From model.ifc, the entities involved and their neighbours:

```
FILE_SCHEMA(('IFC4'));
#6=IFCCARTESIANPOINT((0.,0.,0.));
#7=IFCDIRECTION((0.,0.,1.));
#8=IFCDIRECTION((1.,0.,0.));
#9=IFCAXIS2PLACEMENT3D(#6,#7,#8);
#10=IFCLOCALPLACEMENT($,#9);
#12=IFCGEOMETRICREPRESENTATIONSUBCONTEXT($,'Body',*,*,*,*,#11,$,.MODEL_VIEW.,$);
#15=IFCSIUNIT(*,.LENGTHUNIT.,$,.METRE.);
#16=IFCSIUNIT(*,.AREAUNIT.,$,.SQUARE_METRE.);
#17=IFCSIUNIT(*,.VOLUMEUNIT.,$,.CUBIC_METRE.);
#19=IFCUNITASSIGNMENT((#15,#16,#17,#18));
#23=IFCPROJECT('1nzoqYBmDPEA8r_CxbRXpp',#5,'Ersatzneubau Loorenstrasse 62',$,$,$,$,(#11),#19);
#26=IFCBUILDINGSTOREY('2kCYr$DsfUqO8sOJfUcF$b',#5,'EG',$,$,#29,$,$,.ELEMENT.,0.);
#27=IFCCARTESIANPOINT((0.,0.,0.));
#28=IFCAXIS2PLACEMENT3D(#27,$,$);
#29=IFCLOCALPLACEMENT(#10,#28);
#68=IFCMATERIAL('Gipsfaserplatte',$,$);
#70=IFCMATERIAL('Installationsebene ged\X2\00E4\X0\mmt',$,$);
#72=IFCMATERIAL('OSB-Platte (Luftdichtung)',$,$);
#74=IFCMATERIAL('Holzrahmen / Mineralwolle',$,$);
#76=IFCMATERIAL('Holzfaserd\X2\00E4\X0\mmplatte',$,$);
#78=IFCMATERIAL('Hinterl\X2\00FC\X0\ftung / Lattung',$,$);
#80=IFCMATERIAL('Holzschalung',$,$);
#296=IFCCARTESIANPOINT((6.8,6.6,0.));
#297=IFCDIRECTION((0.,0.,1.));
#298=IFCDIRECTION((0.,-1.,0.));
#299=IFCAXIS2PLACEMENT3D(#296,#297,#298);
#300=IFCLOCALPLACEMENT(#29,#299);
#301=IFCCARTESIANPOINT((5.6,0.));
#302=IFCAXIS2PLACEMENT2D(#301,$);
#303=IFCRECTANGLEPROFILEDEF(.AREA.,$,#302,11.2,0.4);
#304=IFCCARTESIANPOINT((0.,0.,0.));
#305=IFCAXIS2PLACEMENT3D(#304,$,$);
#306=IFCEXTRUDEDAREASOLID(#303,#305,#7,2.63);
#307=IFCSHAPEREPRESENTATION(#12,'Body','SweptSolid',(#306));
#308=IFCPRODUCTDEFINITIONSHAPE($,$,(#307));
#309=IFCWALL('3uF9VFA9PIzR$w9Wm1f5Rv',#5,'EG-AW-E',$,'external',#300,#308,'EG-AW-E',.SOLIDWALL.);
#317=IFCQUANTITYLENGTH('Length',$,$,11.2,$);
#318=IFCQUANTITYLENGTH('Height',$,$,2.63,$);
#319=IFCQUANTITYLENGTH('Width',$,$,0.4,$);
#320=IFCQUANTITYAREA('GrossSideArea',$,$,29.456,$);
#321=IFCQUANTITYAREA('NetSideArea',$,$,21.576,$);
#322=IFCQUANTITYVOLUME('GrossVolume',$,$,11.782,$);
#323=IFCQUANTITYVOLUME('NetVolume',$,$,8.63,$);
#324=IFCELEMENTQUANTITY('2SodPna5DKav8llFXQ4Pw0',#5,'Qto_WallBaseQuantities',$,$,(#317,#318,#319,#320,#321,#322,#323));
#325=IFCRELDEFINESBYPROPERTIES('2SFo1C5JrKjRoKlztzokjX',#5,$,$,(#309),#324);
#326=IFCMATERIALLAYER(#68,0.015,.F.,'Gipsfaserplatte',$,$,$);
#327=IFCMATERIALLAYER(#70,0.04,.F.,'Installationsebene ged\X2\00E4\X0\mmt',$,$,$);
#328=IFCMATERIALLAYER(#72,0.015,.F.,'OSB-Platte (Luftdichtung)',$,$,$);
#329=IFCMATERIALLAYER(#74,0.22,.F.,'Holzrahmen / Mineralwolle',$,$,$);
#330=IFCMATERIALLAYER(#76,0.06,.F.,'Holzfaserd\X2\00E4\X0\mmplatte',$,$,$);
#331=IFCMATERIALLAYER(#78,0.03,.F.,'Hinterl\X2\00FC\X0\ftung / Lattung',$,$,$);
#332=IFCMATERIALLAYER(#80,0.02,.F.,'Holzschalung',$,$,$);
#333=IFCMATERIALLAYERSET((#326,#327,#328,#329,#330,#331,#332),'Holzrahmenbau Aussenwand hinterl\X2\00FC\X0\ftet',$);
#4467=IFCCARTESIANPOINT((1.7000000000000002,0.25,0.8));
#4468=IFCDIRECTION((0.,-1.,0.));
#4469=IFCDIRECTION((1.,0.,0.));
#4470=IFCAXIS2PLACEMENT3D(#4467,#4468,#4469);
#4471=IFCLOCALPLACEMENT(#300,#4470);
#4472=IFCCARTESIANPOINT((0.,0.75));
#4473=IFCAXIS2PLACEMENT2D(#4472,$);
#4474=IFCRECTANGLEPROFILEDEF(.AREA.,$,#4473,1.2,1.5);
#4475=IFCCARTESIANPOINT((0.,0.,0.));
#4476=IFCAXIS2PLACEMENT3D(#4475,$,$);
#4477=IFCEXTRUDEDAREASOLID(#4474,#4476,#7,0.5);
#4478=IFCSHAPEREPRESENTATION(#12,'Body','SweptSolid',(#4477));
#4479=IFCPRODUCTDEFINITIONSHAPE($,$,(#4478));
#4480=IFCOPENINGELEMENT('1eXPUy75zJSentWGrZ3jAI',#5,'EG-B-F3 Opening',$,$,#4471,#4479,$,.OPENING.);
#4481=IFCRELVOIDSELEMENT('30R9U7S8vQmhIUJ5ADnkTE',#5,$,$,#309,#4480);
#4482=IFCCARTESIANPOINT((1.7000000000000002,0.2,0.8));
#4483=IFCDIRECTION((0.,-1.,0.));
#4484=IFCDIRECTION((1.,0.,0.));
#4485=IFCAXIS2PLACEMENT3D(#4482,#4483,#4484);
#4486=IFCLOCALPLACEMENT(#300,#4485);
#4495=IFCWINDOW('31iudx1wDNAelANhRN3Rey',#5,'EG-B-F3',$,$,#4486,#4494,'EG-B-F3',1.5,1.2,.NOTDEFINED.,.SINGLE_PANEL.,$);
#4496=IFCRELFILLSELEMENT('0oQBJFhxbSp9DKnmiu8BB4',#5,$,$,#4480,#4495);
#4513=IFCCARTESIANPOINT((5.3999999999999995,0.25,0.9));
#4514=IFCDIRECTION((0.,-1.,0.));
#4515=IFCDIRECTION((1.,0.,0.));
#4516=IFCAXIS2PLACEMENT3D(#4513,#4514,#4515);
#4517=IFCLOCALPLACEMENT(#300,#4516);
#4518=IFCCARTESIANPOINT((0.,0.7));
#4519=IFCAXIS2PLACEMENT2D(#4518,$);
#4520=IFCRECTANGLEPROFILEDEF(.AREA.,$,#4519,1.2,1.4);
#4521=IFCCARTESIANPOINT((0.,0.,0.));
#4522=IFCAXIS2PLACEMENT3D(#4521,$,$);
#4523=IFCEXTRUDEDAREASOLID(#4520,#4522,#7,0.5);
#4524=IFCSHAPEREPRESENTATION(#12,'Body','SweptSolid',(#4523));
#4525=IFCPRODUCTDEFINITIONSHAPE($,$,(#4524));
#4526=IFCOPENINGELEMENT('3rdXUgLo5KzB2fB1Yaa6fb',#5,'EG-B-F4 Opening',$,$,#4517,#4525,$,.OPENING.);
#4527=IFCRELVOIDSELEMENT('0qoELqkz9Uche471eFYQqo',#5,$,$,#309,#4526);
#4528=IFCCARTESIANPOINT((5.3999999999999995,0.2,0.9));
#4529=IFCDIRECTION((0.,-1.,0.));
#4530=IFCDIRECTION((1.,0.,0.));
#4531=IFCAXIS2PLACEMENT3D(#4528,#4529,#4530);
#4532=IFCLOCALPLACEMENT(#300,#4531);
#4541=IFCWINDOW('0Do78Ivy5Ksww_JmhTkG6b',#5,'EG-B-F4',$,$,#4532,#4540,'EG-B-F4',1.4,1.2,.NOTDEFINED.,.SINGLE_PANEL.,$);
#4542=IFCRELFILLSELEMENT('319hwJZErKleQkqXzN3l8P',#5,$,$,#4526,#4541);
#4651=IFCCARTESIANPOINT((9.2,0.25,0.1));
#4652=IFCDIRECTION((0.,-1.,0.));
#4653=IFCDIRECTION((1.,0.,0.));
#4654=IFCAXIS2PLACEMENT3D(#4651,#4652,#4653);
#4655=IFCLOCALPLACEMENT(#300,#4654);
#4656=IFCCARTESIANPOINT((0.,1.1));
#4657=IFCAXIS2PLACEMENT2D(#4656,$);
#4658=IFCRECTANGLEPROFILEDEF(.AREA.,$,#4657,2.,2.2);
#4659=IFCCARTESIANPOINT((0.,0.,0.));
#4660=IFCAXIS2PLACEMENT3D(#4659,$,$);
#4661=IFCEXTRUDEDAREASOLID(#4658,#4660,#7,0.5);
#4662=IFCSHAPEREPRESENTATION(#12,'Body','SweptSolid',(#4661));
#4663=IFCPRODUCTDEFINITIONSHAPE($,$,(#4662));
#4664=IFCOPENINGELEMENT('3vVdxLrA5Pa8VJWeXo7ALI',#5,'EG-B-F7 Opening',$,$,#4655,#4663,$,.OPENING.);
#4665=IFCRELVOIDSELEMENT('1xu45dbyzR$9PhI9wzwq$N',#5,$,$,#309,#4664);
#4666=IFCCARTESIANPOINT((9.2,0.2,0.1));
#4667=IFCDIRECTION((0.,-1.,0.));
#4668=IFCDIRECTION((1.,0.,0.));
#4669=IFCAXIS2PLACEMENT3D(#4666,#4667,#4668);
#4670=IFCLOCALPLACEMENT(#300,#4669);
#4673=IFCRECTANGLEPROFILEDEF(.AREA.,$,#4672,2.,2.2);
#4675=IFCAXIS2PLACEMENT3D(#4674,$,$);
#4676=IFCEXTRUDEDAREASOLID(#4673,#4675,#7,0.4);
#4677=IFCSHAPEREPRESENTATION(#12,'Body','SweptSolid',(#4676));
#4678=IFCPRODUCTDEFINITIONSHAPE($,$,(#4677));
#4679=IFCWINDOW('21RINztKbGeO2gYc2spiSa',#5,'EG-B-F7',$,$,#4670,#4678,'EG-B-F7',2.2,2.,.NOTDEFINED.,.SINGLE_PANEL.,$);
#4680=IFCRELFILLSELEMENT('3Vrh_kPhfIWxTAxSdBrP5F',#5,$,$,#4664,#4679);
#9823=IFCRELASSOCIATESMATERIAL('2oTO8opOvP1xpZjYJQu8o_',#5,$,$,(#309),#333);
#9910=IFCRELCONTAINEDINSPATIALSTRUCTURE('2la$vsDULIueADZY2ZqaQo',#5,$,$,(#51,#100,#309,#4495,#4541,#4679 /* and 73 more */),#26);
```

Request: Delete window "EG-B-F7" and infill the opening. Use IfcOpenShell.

```python
import ifcopenshell
import ifcopenshell.api.feature
import ifcopenshell.api.pset
import ifcopenshell.api.root
import ifcopenshell.geom
import ifcopenshell.util.element
import ifcopenshell.util.shape
import ifcopenshell.util.unit

model = ifcopenshell.open("model.ifc")
area_scale = ifcopenshell.util.unit.calculate_unit_scale(model, "AREAUNIT")
volume_scale = ifcopenshell.util.unit.calculate_unit_scale(model, "VOLUMEUNIT")
settings = ifcopenshell.geom.settings()


def volume(element):
    """Net volume in cubic metres, openings subtracted."""
    shape = ifcopenshell.geom.create_shape(settings, element)
    return ifcopenshell.util.shape.get_volume(shape.geometry)


window = model.by_id(4679)
opening = window.FillsVoids[0].RelatingOpeningElement
wall = opening.VoidsElements[0].RelatingBuildingElement
before = volume(wall)

ifcopenshell.api.root.remove_product(model, product=window)
ifcopenshell.api.feature.remove_feature(model, feature=opening)

after = volume(wall)
thickness = 0.4  # wall thickness in metres

# Update the wall's stored quantities.
qto = model.by_id(ifcopenshell.util.element.get_pset(wall, "Qto_WallBaseQuantities", should_inherit=False)["id"])
ifcopenshell.api.pset.edit_qto(model, qto=qto, properties={
    "NetSideArea": after / thickness / area_scale,
    "NetVolume": after / volume_scale,
})

print(f"wall volume {before:.3f} -> {after:.3f} m3")

model.write("model_rev.ifc")
```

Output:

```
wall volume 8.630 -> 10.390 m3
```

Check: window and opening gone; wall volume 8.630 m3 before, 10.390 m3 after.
